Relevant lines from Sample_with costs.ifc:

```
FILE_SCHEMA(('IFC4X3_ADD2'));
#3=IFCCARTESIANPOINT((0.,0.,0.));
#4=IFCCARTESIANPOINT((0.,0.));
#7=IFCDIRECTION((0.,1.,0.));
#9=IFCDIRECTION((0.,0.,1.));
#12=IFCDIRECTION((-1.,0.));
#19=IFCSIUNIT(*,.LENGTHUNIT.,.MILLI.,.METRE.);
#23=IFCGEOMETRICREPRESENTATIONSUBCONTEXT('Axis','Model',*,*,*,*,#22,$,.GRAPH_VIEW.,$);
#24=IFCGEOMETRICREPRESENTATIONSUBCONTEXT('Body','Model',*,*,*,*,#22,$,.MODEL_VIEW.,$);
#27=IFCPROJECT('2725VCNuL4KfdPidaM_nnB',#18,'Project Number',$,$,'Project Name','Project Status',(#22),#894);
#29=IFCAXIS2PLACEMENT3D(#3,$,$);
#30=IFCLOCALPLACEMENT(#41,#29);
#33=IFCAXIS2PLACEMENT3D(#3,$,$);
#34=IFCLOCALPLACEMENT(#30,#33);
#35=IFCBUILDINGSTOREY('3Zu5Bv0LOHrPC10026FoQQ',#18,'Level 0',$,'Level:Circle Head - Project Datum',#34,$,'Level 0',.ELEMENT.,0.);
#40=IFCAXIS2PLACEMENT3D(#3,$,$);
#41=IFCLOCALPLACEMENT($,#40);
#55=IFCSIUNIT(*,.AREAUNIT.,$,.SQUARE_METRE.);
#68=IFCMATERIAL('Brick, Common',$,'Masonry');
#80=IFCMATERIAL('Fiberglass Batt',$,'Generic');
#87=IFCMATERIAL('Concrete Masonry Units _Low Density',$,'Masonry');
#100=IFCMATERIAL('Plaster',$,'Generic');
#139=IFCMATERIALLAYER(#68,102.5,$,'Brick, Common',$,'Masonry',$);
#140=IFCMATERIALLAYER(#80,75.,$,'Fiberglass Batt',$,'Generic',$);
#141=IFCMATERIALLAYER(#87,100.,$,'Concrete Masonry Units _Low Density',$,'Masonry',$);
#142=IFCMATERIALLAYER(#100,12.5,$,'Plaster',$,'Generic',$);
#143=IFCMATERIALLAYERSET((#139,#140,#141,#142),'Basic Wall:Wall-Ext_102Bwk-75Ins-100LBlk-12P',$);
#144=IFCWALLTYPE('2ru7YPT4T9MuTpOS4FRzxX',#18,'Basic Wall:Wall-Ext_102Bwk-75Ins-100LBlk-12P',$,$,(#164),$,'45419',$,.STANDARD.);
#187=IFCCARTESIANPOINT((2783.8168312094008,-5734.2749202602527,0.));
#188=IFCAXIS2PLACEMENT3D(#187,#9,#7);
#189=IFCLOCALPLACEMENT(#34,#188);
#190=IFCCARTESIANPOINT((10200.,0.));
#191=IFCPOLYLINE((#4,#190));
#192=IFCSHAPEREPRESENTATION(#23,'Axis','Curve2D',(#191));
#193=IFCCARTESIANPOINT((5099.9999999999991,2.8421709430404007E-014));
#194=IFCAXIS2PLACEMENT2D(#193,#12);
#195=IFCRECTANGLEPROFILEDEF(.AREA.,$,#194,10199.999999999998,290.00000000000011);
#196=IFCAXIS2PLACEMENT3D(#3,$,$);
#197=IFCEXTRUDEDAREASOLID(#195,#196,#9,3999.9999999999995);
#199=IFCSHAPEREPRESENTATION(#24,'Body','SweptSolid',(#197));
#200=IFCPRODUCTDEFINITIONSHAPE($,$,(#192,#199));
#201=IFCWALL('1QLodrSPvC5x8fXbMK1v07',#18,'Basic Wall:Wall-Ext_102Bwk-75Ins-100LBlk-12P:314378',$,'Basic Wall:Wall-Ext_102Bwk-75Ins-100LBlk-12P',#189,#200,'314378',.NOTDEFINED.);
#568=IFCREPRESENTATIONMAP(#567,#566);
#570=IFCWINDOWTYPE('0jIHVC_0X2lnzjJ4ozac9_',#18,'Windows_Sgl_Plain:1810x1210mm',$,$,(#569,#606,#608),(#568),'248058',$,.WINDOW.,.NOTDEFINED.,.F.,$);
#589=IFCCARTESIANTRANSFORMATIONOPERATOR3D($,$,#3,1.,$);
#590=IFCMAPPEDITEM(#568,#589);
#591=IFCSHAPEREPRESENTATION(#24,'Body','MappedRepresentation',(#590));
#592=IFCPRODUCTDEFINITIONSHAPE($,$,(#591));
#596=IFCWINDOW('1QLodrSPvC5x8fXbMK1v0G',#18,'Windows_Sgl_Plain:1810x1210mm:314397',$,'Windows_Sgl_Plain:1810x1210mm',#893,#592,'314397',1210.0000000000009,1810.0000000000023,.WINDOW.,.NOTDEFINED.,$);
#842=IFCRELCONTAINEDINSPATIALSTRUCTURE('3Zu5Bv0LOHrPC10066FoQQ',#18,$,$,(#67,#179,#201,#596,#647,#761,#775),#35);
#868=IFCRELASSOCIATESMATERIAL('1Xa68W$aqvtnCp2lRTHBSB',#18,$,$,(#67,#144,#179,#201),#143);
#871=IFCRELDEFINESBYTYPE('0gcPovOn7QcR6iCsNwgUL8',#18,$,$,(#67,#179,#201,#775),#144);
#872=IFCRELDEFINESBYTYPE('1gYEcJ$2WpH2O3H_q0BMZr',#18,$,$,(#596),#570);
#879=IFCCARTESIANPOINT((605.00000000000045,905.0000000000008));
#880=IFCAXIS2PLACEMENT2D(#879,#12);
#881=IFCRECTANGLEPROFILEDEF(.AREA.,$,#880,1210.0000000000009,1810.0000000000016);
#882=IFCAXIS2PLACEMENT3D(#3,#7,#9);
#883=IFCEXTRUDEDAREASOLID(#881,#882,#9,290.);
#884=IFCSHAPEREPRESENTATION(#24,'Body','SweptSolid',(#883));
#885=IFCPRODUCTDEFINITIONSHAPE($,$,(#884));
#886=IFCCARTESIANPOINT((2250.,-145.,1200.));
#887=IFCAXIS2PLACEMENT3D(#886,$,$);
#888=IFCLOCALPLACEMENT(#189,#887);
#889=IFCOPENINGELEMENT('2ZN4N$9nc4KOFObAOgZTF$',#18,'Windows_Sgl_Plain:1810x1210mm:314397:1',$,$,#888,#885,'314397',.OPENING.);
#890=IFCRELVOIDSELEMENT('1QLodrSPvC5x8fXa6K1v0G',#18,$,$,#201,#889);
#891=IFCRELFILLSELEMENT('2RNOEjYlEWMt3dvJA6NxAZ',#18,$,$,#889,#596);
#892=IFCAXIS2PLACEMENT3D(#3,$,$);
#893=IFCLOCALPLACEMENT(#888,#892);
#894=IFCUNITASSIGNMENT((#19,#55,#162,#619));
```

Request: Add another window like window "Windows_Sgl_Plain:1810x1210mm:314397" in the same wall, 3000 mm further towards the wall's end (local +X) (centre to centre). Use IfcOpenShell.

```python
import ifcopenshell
import ifcopenshell.api.feature
import ifcopenshell.api.geometry
import ifcopenshell.api.root
import ifcopenshell.geom
import ifcopenshell.util.element
import ifcopenshell.util.placement
import ifcopenshell.util.shape
import ifcopenshell.util.unit

model = ifcopenshell.open("Sample_with costs.ifc")
unit_scale = ifcopenshell.util.unit.calculate_unit_scale(model)
settings = ifcopenshell.geom.settings()


def volume(element):
    """Net volume in cubic metres, openings subtracted."""
    shape = ifcopenshell.geom.create_shape(settings, element)
    return ifcopenshell.util.shape.get_volume(shape.geometry)


def reuse_history(source, copy):
    """copy_class also copies each property set's owner history, people and application; keep the originals."""
    for rel in copy.IsDefinedBy:
        if rel.is_a("IfcRelDefinesByProperties") and (history := rel.RelatingPropertyDefinition.OwnerHistory):
            rel.RelatingPropertyDefinition.OwnerHistory = source.OwnerHistory
            ifcopenshell.util.element.remove_deep2(model, history)


window = model.by_guid("1QLodrSPvC5x8fXbMK1v0G")
opening = window.FillsVoids[0].RelatingOpeningElement
wall = opening.VoidsElements[0].RelatingBuildingElement
before = volume(wall)
shift = ifcopenshell.util.placement.get_local_placement(wall.ObjectPlacement)[:3, 0] * 3 / unit_scale

# copy_class copies the void relationship, type, container and properties, but no geometry.
new_opening = ifcopenshell.api.root.copy_class(model, product=opening)
new_opening.Representation = ifcopenshell.util.element.copy_deep(
    model, opening.Representation, exclude=["IfcGeometricRepresentationContext", "IfcRepresentationMap"]
)
new_opening.Name = "Windows_Sgl_Plain:1810x1210mm"
new_opening.Tag = None
new_window = ifcopenshell.api.root.copy_class(model, product=window)
new_window.Representation = ifcopenshell.util.element.copy_deep(
    model, window.Representation, exclude=["IfcGeometricRepresentationContext", "IfcRepresentationMap"]
)
new_window.Name = "Windows_Sgl_Plain:1810x1210mm"
new_window.Tag = None
reuse_history(window, new_window)
ifcopenshell.api.feature.add_filling(model, opening=new_opening, element=new_window)

for old, new in ((opening, new_opening), (window, new_window)):
    matrix = ifcopenshell.util.placement.get_local_placement(old.ObjectPlacement)
    matrix[:3, 3] += shift
    ifcopenshell.api.geometry.edit_object_placement(model, product=new, matrix=matrix, is_si=False)

after = volume(wall)

print(f"wall volume {before:.3f} -> {after:.3f} m3")

model.write("Sample_with costs_updated.ifc")
```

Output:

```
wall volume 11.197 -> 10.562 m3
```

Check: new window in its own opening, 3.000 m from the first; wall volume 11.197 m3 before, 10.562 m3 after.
